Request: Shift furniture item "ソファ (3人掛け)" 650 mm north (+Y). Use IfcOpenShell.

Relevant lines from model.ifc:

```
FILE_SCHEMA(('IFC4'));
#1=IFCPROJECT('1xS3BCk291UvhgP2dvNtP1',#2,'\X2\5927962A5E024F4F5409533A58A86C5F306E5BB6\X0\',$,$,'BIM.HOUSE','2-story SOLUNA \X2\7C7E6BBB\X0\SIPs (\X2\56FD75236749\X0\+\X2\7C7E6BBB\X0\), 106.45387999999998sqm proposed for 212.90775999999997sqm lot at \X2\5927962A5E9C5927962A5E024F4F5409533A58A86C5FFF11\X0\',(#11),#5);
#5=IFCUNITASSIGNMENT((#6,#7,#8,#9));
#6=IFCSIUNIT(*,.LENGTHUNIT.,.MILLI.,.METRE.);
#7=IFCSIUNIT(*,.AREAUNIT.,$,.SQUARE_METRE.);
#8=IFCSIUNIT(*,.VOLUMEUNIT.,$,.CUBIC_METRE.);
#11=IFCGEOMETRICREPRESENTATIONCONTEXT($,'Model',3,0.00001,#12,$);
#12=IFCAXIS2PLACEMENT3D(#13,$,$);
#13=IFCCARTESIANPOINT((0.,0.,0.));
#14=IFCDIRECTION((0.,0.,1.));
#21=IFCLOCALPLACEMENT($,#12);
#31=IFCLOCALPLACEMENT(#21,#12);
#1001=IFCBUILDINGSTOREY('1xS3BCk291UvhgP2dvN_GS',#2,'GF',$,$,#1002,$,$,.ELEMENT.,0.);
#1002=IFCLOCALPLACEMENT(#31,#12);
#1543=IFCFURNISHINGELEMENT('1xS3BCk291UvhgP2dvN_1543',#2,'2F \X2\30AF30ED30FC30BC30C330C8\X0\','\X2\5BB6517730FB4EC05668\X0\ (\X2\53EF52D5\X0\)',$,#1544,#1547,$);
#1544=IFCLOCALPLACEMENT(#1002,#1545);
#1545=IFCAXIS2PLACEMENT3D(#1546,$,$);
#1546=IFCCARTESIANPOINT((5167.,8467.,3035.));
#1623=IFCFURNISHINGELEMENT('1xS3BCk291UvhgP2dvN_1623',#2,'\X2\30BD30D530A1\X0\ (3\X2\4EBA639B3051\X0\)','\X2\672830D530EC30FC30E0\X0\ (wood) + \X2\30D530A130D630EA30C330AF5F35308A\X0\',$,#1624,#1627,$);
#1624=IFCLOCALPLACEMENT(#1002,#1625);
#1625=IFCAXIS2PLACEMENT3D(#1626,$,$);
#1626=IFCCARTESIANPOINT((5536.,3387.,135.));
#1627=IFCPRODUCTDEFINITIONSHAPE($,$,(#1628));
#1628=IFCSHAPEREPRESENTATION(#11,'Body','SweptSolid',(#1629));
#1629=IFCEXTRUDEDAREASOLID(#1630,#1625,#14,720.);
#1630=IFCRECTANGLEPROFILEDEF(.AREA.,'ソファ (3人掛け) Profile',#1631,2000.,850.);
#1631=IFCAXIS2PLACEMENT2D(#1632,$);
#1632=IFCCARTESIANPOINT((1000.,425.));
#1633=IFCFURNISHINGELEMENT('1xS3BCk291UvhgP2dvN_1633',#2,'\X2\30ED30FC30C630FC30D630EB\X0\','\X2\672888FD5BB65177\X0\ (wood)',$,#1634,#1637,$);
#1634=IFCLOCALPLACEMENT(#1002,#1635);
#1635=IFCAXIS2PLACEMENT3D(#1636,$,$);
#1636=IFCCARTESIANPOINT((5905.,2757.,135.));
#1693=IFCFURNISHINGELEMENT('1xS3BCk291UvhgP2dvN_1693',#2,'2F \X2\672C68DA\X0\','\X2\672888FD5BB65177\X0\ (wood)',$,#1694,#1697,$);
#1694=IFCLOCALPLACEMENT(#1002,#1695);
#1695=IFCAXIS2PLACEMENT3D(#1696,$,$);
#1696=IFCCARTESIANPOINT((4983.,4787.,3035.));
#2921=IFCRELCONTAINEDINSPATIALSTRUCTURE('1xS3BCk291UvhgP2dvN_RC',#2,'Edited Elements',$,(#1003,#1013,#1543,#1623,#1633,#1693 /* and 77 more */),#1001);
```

```python
import ifcopenshell
import ifcopenshell.api.geometry
import ifcopenshell.util.placement
import ifcopenshell.util.unit

model = ifcopenshell.open("model.ifc")
unit_scale = ifcopenshell.util.unit.calculate_unit_scale(model)

item = model.by_id(1623)
matrix = ifcopenshell.util.placement.get_local_placement(item.ObjectPlacement)
matrix[1, 3] += 0.65 / unit_scale
ifcopenshell.api.geometry.edit_object_placement(model, product=item, matrix=matrix, is_si=False)

print(ifcopenshell.util.placement.get_local_placement(item.ObjectPlacement).round(3) + 0.0)

model.write("model_updated.ifc")
```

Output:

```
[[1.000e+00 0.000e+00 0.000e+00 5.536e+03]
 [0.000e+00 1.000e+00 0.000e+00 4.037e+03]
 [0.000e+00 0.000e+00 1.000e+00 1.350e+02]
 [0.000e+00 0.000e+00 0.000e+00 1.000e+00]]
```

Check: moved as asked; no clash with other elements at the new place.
